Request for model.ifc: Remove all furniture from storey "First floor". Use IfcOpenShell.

First a look at what the model holds.

```python
import ifcopenshell
import ifcopenshell.util.element

model = ifcopenshell.open("model.ifc")
print(model.schema)
storey = next(s for s in model.by_type("IfcBuildingStorey") if s.Name == "First floor")
furniture = [e for e in ifcopenshell.util.element.get_decomposition(storey) if e.is_a("IfcFurnishingElement")]
seen = {}
for e in furniture:
    element_type = ifcopenshell.util.element.get_type(e)
    name = element_type.Name if element_type not in (None, e) else None
    seen[name] = seen.get(name, 0) + 1
for name, count in sorted(seen.items(), key=str):
    print(count, "x", name)
```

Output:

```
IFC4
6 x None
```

```python
import ifcopenshell
import ifcopenshell.api.root
import ifcopenshell.util.element

model = ifcopenshell.open("model.ifc")

storey = next(s for s in model.by_type("IfcBuildingStorey") if s.Name == "First floor")
furniture = [e for e in ifcopenshell.util.element.get_decomposition(storey) if e.is_a("IfcFurnishingElement")]

for e in furniture:
    ifcopenshell.api.root.remove_product(model, product=e)
print(len(furniture), "removed")

model.write("model-out.ifc")
```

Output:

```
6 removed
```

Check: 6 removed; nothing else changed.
